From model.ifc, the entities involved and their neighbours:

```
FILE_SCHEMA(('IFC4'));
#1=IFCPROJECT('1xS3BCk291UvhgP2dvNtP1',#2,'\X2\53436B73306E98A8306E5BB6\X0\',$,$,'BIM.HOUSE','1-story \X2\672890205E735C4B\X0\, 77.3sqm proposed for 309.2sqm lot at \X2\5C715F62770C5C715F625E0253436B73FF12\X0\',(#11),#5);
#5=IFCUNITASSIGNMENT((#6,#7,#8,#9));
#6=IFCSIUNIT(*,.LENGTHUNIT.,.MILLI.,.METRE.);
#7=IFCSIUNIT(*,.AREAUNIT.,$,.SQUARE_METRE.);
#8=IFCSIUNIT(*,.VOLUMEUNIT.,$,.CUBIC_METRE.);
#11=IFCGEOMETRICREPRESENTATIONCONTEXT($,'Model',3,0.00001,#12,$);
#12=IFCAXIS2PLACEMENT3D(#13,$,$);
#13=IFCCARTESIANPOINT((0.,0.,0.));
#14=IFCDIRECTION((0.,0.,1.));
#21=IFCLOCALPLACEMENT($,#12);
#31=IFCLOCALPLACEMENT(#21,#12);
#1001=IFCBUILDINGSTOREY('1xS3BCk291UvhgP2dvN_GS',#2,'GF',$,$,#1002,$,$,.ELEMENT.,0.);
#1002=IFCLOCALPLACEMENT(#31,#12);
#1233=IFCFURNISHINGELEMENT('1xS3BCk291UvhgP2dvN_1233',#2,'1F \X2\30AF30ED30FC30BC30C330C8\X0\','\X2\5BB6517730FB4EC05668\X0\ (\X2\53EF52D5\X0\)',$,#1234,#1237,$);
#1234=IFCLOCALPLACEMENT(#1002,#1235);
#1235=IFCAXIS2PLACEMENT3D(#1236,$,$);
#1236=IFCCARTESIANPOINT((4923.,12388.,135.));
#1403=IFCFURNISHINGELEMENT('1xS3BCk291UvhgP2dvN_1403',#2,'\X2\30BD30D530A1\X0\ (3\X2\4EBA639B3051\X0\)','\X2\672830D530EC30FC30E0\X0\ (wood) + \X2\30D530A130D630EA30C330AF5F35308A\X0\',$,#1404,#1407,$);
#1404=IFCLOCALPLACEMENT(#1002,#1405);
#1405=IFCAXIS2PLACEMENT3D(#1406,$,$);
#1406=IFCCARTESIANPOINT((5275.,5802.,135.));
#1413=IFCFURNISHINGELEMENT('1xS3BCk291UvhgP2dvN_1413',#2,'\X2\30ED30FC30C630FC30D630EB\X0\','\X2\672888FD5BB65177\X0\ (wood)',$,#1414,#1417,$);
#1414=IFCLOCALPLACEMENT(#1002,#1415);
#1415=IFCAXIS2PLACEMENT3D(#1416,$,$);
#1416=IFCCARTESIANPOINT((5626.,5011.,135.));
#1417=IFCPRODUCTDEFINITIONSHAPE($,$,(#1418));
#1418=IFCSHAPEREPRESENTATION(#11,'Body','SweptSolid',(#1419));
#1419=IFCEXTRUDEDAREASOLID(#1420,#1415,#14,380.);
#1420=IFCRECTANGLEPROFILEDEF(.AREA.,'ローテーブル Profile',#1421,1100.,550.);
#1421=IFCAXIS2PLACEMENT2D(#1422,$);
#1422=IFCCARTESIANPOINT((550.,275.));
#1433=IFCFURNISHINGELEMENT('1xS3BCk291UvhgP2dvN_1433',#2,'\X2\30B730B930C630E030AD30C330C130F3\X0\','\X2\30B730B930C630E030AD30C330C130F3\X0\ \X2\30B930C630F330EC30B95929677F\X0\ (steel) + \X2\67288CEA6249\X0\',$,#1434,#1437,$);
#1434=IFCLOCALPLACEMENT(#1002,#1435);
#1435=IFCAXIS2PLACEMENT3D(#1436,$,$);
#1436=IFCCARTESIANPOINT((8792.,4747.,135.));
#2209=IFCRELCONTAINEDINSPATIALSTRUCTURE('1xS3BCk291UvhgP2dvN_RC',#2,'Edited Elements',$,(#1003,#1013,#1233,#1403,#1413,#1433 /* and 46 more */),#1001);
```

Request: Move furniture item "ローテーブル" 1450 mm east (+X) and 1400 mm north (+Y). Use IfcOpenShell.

```python
import ifcopenshell
import ifcopenshell.api.geometry
import ifcopenshell.util.placement

model = ifcopenshell.open("model.ifc")

item = model.by_guid("1xS3BCk291UvhgP2dvN_1413")
matrix = ifcopenshell.util.placement.get_local_placement(item.ObjectPlacement)
matrix[0, 3] += 1450.0
matrix[1, 3] += 1400.0
ifcopenshell.api.geometry.edit_object_placement(model, product=item, matrix=matrix, is_si=False)

print(ifcopenshell.util.placement.get_local_placement(item.ObjectPlacement).round(3) + 0.0)

model.write("model_rev.ifc")
```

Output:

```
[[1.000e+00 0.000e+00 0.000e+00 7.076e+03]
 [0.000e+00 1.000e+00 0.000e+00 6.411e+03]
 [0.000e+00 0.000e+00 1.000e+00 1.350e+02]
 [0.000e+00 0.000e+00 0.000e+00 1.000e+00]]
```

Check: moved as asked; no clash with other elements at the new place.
